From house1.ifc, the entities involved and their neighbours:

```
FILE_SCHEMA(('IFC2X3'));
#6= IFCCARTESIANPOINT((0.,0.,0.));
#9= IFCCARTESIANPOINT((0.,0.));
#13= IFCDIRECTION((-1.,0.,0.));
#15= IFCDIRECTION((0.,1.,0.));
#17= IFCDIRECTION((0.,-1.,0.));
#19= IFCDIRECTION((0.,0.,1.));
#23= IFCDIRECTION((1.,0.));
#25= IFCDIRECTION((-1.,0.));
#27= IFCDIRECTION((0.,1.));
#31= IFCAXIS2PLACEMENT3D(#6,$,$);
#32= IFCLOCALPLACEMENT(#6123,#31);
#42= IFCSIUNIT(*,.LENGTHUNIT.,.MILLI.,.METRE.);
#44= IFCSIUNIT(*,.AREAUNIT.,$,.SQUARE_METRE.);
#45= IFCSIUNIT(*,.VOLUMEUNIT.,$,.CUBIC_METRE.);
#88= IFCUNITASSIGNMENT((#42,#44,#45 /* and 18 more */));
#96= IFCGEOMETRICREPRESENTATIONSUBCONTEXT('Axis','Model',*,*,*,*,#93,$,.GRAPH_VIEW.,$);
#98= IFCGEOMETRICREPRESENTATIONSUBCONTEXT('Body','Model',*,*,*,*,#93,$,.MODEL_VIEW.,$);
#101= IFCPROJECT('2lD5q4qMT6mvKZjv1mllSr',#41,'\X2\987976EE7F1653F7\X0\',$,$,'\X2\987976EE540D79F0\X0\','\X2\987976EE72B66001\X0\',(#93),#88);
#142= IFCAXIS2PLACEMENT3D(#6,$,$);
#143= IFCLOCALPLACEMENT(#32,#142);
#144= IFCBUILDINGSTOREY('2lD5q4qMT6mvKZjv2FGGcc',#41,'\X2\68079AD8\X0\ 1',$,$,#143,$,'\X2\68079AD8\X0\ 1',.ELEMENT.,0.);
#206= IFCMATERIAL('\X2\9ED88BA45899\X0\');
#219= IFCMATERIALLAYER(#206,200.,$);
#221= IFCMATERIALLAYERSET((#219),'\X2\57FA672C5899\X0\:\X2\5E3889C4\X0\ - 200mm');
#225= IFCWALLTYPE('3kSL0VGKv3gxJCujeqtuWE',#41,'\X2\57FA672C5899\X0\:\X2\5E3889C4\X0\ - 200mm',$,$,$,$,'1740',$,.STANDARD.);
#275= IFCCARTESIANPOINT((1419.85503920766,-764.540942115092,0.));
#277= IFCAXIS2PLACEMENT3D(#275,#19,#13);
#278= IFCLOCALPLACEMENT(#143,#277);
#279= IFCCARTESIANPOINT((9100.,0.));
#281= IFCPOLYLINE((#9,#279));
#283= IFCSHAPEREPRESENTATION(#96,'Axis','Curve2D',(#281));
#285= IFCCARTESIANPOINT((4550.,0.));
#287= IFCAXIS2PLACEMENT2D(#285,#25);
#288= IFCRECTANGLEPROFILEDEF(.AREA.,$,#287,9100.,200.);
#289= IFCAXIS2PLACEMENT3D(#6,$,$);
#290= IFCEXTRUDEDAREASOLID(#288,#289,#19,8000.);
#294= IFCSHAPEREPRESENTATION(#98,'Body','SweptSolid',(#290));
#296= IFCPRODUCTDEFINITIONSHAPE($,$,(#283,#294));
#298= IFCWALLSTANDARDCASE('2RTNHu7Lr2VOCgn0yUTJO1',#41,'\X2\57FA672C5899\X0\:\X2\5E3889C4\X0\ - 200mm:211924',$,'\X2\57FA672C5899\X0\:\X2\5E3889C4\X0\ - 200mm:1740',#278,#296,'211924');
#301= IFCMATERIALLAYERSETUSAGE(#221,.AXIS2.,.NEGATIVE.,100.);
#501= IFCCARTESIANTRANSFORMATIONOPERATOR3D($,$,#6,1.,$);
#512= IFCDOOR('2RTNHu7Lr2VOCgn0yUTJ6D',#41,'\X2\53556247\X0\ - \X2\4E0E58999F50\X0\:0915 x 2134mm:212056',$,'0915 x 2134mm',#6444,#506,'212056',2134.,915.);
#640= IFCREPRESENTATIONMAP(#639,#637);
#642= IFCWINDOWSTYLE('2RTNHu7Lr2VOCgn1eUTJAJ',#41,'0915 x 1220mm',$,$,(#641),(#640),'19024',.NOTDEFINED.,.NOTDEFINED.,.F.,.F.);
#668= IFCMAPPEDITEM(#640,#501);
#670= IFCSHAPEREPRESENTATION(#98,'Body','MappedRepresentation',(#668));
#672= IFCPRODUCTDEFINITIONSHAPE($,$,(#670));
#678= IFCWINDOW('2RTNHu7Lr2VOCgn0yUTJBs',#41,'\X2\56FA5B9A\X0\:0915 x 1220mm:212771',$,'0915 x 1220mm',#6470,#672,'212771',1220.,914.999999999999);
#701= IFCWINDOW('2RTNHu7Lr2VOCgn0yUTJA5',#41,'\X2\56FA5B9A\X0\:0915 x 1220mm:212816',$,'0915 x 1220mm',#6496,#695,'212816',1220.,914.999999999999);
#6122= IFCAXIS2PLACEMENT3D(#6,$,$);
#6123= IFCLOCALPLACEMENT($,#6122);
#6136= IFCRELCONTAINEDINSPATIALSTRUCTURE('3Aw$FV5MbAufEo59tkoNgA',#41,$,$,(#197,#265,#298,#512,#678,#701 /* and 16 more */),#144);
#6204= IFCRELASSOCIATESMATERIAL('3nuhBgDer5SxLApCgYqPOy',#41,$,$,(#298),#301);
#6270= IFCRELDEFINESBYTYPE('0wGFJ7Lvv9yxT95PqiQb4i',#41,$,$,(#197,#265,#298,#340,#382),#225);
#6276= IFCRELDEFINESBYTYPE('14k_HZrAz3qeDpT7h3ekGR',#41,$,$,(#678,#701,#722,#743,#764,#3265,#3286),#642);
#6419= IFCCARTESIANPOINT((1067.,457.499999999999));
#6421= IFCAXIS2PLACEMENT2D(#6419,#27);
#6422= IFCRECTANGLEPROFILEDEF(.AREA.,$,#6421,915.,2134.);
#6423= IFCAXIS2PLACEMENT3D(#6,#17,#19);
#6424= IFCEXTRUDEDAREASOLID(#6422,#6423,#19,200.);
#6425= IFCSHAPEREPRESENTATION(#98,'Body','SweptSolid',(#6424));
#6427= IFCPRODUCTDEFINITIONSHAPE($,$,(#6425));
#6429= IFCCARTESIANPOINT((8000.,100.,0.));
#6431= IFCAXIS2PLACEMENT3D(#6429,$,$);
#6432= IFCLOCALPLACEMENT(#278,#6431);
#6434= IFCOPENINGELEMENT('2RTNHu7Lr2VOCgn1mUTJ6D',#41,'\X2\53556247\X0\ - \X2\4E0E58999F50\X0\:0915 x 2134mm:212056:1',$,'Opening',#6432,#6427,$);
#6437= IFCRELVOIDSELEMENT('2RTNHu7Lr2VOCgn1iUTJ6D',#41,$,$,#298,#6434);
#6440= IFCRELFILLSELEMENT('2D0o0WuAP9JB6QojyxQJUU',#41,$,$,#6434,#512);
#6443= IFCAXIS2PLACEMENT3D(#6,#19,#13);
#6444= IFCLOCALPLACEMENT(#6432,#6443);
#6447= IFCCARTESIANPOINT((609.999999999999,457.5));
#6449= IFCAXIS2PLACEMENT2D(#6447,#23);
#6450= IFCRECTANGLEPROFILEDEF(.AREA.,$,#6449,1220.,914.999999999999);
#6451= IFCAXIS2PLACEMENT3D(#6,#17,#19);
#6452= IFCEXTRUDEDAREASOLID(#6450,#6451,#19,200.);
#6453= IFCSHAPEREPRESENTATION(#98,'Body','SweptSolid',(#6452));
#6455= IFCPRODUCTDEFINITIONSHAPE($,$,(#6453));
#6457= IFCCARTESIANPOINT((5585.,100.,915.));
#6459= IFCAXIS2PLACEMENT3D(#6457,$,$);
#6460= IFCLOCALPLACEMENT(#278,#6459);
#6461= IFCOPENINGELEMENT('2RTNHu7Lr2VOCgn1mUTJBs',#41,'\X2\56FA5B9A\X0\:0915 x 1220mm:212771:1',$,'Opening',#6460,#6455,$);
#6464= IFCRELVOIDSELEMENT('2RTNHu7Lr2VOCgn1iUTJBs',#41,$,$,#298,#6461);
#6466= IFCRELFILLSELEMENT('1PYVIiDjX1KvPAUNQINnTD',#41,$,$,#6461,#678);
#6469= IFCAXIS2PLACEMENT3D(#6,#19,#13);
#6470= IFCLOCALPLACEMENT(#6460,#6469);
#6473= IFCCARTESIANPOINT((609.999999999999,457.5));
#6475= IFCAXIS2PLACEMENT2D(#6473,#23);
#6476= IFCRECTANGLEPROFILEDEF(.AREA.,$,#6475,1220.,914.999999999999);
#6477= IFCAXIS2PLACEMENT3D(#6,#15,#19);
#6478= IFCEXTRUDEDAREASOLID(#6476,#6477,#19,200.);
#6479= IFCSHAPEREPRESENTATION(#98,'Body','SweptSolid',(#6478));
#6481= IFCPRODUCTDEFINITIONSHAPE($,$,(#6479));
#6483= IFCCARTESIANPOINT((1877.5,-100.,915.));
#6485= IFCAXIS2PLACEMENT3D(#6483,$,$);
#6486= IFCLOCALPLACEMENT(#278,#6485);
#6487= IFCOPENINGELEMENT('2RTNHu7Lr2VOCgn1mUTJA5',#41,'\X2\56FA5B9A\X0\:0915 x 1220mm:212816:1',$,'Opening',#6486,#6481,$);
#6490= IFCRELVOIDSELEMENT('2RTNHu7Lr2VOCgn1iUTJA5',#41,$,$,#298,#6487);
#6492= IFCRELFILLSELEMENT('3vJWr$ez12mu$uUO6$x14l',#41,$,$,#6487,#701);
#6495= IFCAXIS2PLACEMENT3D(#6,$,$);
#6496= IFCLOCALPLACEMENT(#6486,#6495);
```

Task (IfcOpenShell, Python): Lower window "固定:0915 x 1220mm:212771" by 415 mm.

```python
import numpy as np
import ifcopenshell
import ifcopenshell.api.geometry
import ifcopenshell.util.placement
import ifcopenshell.util.unit

model = ifcopenshell.open("house1.ifc")
unit_scale = ifcopenshell.util.unit.calculate_unit_scale(model)

window = model.by_guid("2RTNHu7Lr2VOCgn0yUTJBs")
opening = window.FillsVoids[0].RelatingOpeningElement
dz = -415.0

shift = np.array([0.0, 0.0, dz])
# The window is placed relative to its opening, so it follows when the opening moves.
matrix = ifcopenshell.util.placement.get_local_placement(opening.ObjectPlacement)
matrix[:3, 3] += shift
ifcopenshell.api.geometry.edit_object_placement(
    model, product=opening, matrix=matrix, is_si=False, should_transform_children=True
)

print(f"moved by {dz * unit_scale:+.3f} m")

model.write("house1_rev.ifc")
```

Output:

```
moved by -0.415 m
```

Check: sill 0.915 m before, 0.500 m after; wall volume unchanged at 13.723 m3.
